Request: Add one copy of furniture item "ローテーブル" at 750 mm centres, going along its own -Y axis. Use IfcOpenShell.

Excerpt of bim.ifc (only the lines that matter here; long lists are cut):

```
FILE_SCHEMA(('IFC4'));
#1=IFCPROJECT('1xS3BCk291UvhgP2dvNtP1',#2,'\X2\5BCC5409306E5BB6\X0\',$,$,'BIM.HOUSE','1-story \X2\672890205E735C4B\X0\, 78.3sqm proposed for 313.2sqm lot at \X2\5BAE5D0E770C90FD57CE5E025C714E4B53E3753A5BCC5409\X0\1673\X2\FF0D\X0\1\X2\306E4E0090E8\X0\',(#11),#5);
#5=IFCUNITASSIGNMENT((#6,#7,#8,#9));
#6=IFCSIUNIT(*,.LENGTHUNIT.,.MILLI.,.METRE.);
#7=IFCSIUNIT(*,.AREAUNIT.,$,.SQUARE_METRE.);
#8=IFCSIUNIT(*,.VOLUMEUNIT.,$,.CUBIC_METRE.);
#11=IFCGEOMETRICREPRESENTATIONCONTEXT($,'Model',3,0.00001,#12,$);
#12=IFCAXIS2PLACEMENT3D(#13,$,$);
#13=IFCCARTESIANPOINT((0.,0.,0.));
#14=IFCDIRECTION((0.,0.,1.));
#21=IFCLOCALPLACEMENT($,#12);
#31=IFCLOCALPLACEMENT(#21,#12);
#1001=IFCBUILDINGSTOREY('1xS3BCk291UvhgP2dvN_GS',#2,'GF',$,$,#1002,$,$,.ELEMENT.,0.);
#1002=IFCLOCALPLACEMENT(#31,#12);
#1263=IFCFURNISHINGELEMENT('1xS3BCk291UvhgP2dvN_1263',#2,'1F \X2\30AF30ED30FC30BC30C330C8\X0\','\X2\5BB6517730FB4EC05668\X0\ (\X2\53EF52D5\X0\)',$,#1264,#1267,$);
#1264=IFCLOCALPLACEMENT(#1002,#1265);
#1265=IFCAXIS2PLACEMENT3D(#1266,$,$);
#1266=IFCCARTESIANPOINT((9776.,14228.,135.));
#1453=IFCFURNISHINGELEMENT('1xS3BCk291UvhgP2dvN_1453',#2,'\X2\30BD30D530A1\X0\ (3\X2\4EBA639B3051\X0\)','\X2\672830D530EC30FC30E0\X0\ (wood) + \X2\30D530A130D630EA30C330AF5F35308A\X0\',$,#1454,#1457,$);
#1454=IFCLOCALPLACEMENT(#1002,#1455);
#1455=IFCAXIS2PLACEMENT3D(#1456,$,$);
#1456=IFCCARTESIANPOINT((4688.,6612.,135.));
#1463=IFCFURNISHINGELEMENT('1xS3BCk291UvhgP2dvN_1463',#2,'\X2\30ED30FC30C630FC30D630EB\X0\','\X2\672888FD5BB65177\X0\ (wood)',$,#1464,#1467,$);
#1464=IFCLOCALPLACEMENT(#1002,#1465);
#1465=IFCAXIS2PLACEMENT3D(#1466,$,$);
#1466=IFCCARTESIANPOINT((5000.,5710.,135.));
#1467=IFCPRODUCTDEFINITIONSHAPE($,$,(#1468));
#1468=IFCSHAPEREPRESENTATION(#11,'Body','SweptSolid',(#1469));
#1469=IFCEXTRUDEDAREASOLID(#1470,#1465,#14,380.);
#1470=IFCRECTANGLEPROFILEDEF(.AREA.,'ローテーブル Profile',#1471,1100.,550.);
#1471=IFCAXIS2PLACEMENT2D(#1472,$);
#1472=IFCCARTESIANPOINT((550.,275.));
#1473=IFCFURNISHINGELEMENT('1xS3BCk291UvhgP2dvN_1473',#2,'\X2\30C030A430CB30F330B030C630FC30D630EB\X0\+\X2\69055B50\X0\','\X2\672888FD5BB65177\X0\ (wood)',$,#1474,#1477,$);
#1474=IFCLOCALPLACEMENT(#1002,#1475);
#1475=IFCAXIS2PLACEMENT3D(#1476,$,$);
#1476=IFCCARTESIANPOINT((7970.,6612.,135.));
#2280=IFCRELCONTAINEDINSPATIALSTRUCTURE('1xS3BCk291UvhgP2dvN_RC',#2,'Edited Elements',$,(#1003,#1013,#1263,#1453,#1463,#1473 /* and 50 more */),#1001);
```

```python
import ifcopenshell
import ifcopenshell.api.geometry
import ifcopenshell.api.root
import ifcopenshell.util.element
import ifcopenshell.util.placement

model = ifcopenshell.open("bim.ifc")


def reuse_history(source, copy):
    """copy_class also copies each property set's owner history, people and application; keep the originals."""
    for rel in copy.IsDefinedBy:
        if rel.is_a("IfcRelDefinesByProperties") and (history := rel.RelatingPropertyDefinition.OwnerHistory):
            rel.RelatingPropertyDefinition.OwnerHistory = source.OwnerHistory
            ifcopenshell.util.element.remove_deep2(model, history)


source = model.by_id(1463)
base = ifcopenshell.util.placement.get_local_placement(source.ObjectPlacement)
step = -base[:3, 1] * 750.0

for i in range(1, 2):
    copy = ifcopenshell.api.root.copy_class(model, product=source)
    copy.Representation = ifcopenshell.util.element.copy_deep(
        model, source.Representation, exclude=["IfcGeometricRepresentationContext", "IfcRepresentationMap"]
    )
    reuse_history(source, copy)
    matrix = base.copy()
    matrix[:3, 3] += i * step
    print("added at", matrix[:3, 3].round(3) + 0.0)
    ifcopenshell.api.geometry.edit_object_placement(model, product=copy, matrix=matrix, is_si=False)

model.write("bim_rev.ifc")
```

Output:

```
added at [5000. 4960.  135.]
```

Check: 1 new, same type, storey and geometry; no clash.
